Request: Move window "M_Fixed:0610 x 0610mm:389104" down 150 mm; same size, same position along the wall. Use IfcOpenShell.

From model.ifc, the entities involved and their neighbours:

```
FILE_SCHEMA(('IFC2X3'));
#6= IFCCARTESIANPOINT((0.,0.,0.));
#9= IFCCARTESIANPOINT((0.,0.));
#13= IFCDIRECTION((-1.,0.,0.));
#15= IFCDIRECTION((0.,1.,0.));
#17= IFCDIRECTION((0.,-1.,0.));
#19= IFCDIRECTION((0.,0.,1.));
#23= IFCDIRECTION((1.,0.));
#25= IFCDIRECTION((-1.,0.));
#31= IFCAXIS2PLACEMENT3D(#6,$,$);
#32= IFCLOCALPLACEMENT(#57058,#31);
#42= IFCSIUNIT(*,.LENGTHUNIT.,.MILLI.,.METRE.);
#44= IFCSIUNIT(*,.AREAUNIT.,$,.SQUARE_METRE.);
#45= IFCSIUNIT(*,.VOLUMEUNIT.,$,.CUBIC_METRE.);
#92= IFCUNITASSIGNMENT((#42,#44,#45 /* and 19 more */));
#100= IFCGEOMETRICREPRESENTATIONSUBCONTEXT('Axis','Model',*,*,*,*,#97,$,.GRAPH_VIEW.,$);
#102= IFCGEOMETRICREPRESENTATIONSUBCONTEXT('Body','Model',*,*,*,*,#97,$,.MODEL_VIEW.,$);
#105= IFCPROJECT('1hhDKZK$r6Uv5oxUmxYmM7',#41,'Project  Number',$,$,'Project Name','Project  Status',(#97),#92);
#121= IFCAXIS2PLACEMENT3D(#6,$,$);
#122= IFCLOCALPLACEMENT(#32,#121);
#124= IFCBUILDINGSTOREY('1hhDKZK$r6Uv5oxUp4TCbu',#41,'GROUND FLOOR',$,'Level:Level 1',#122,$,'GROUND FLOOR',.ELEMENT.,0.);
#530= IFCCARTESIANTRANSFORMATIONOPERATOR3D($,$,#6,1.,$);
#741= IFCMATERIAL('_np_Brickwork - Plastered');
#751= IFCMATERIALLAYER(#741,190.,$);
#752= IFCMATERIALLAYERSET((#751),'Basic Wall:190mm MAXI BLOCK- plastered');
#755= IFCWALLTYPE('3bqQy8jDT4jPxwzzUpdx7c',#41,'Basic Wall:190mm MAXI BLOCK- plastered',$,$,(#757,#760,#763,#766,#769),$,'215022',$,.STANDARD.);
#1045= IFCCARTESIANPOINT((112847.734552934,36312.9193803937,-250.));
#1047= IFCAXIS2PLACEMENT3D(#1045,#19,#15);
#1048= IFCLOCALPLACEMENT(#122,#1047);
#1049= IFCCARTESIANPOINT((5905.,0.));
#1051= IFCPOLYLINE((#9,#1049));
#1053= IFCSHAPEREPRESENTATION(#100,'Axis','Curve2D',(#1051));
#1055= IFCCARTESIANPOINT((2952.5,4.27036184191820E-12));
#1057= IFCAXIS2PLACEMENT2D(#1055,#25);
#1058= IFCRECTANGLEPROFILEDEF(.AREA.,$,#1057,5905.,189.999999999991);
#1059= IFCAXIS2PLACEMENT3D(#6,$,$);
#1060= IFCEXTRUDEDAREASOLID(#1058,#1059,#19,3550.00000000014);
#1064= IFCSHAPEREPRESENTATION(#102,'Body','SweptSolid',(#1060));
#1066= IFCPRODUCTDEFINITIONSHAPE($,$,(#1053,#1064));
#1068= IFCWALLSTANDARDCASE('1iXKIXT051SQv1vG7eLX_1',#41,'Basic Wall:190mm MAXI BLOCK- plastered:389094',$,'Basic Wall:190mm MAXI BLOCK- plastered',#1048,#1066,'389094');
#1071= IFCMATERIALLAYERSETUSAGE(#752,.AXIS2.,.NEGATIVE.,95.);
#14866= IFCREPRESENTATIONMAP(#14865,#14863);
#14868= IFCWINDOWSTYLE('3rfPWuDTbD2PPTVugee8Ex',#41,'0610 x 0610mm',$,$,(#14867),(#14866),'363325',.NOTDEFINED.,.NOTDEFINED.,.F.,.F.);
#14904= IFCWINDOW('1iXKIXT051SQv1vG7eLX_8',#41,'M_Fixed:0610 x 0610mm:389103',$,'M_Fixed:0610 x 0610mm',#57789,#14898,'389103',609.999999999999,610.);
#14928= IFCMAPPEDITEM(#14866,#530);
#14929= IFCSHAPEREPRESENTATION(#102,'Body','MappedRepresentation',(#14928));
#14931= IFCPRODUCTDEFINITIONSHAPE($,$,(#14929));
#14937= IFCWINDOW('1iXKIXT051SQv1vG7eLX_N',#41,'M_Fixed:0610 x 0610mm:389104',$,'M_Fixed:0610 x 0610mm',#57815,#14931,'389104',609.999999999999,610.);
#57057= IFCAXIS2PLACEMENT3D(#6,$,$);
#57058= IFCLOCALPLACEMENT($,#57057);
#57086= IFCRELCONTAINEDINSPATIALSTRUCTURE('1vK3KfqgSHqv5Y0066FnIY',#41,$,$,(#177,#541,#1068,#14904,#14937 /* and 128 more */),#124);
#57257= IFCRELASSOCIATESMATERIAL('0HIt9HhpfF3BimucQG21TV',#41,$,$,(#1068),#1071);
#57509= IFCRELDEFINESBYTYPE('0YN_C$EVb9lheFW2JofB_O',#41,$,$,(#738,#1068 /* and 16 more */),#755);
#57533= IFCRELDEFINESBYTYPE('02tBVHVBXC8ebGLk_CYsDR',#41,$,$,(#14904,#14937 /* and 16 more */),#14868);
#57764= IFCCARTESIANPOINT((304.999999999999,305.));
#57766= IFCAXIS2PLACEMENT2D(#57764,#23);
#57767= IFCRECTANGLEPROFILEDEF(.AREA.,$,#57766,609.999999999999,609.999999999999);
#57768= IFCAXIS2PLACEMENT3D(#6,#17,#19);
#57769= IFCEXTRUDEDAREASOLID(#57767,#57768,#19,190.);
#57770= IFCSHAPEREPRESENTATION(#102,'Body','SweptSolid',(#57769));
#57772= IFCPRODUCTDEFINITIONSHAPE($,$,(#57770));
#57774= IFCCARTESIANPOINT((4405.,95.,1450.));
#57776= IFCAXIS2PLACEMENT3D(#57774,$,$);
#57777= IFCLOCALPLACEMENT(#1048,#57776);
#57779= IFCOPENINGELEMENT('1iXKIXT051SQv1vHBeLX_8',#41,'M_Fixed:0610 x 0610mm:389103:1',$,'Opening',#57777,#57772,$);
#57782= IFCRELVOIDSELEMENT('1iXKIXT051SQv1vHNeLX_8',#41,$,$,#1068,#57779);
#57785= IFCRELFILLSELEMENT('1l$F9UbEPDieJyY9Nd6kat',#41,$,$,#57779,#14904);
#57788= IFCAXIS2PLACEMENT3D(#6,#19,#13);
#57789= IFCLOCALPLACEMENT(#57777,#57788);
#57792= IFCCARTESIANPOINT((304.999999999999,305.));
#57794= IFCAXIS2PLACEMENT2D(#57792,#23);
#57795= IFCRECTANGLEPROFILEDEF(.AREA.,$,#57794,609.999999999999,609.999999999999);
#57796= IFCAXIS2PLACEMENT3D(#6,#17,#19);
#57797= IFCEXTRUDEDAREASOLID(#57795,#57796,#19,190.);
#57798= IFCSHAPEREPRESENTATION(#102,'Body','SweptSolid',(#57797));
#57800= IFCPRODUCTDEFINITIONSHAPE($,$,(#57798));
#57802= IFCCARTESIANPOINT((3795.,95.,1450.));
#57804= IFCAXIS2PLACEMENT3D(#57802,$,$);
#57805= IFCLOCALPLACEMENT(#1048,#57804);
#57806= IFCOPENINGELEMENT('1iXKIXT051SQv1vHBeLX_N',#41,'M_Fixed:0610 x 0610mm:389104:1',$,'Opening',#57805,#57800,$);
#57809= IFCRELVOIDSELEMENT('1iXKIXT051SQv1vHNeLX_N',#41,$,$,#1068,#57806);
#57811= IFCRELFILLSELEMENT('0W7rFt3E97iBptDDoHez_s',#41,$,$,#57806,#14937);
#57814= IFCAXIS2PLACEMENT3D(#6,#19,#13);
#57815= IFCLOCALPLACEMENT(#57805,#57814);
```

```python
import numpy as np
import ifcopenshell
import ifcopenshell.api.geometry
import ifcopenshell.util.placement
import ifcopenshell.util.unit

model = ifcopenshell.open("model.ifc")
unit_scale = ifcopenshell.util.unit.calculate_unit_scale(model)

window = model.by_id(14937)
opening = window.FillsVoids[0].RelatingOpeningElement
dz = -0.15 / unit_scale

shift = np.array([0.0, 0.0, dz])
# The window is placed relative to its opening, so it follows when the opening moves.
matrix = ifcopenshell.util.placement.get_local_placement(opening.ObjectPlacement)
matrix[:3, 3] += shift
ifcopenshell.api.geometry.edit_object_placement(
    model, product=opening, matrix=matrix, is_si=False, should_transform_children=True
)

print(f"moved by {dz * unit_scale:+.3f} m")

model.write("model_updated.ifc")
```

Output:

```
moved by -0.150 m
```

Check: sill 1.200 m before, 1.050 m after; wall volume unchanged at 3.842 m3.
